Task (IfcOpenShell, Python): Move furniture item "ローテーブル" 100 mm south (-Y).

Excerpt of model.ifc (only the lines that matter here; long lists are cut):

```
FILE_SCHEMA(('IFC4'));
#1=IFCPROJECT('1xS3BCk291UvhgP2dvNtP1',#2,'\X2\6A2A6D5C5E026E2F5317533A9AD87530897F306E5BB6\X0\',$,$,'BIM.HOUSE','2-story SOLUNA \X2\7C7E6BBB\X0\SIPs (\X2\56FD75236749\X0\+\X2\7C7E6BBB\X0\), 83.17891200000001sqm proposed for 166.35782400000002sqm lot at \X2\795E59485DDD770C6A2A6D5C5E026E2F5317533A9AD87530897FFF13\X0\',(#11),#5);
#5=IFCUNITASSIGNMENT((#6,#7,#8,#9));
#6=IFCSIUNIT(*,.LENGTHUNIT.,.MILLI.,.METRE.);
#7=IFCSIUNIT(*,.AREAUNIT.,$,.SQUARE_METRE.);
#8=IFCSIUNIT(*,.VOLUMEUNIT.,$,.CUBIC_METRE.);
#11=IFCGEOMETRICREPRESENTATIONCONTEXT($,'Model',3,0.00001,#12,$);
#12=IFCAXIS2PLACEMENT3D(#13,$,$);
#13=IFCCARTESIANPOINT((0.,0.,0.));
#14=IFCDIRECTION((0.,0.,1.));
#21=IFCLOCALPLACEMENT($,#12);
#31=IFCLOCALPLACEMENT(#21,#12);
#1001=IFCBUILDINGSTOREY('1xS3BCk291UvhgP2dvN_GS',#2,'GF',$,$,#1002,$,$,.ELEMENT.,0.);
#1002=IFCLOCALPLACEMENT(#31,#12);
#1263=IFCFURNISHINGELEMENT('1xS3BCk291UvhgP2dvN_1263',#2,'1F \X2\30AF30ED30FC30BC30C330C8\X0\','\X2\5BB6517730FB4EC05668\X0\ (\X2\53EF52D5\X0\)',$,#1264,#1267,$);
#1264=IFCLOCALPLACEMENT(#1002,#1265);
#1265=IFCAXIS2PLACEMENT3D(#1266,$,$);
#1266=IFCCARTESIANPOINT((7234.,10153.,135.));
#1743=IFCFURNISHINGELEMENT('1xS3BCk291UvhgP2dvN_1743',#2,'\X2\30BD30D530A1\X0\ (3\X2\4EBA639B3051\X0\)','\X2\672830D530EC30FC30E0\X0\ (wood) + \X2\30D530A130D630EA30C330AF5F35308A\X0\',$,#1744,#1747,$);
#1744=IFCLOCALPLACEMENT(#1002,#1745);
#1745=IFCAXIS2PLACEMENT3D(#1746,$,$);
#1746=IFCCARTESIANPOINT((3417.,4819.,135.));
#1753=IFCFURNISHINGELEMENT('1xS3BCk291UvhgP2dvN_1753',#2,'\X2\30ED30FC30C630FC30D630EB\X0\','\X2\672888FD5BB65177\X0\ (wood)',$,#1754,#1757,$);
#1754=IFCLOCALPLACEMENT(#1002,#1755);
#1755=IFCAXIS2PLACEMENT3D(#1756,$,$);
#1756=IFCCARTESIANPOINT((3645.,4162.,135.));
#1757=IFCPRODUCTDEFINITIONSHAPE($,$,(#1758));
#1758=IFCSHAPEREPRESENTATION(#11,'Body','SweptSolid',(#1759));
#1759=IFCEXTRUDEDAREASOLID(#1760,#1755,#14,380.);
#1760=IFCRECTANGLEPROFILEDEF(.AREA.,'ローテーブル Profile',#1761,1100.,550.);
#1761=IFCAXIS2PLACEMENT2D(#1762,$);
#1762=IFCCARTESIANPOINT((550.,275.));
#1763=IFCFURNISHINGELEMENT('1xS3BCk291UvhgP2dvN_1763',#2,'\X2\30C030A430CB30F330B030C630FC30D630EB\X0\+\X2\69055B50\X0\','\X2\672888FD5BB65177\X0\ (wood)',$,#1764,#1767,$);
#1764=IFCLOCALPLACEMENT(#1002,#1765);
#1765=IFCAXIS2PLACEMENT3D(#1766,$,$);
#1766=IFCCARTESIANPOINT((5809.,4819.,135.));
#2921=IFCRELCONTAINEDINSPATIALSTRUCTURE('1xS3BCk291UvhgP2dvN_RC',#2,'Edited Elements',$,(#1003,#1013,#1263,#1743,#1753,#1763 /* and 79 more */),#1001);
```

```python
import ifcopenshell
import ifcopenshell.api.geometry
import ifcopenshell.util.placement
import ifcopenshell.util.unit

model = ifcopenshell.open("model.ifc")
unit_scale = ifcopenshell.util.unit.calculate_unit_scale(model)

item = model.by_guid("1xS3BCk291UvhgP2dvN_1753")
matrix = ifcopenshell.util.placement.get_local_placement(item.ObjectPlacement)
matrix[1, 3] -= 0.1 / unit_scale
ifcopenshell.api.geometry.edit_object_placement(model, product=item, matrix=matrix, is_si=False)

print(ifcopenshell.util.placement.get_local_placement(item.ObjectPlacement).round(3) + 0.0)

model.write("model_updated.ifc")
```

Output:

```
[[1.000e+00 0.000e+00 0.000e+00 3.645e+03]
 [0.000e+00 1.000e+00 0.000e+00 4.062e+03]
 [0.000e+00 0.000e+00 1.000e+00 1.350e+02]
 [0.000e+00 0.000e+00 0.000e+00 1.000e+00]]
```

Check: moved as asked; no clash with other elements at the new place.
